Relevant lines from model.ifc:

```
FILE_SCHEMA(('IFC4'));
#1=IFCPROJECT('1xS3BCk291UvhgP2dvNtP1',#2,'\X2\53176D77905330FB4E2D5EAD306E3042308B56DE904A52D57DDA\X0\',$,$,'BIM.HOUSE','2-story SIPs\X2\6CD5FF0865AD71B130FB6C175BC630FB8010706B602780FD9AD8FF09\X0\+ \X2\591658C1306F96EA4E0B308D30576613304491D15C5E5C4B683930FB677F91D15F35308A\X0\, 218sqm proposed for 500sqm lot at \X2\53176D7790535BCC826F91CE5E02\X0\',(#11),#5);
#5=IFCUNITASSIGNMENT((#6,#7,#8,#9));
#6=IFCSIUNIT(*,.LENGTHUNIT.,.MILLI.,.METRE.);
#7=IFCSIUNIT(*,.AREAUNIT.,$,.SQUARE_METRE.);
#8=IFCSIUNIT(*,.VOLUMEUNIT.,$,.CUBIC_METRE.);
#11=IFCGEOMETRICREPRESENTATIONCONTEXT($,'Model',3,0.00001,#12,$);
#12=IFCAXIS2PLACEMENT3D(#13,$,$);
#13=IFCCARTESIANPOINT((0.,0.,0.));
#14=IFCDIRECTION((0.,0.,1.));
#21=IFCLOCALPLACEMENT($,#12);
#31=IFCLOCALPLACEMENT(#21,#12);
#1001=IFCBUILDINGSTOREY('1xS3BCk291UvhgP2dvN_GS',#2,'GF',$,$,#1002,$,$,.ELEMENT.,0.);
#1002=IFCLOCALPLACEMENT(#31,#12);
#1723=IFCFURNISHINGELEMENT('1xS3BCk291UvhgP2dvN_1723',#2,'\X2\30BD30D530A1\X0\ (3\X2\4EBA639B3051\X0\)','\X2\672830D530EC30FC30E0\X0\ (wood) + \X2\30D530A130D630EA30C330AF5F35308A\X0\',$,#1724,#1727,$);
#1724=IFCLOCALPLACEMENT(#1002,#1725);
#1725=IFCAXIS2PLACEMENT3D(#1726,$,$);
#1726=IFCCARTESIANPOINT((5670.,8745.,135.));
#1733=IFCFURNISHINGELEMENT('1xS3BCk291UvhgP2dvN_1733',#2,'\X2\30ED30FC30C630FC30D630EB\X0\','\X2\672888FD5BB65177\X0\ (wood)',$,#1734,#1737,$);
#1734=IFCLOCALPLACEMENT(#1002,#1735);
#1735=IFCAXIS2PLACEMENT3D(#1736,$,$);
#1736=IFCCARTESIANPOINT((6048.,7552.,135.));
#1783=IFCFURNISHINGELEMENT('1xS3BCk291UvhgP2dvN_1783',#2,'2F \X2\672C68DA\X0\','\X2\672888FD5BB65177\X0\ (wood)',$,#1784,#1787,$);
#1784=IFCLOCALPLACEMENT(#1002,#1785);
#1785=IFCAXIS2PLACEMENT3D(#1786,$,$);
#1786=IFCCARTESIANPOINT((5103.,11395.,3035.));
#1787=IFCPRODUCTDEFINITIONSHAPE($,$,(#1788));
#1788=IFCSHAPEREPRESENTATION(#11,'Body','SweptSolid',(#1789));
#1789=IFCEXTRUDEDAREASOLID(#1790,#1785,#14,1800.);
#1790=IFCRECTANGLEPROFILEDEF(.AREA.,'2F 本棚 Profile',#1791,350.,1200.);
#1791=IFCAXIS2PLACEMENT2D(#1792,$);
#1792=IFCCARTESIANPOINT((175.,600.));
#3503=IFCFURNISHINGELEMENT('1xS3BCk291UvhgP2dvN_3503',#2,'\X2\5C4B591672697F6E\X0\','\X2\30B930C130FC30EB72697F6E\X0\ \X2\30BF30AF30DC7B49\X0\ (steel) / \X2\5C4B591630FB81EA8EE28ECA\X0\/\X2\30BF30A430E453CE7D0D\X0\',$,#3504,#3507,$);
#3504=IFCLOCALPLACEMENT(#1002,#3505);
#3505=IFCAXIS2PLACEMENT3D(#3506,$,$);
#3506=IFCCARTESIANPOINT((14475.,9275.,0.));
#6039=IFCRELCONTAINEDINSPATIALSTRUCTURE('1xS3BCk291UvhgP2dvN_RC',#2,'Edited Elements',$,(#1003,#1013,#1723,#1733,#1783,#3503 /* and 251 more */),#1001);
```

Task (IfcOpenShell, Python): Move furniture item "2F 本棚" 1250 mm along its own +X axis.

```python
import ifcopenshell
import ifcopenshell.api.geometry
import ifcopenshell.util.placement
import ifcopenshell.util.unit

model = ifcopenshell.open("model.ifc")
unit_scale = ifcopenshell.util.unit.calculate_unit_scale(model)

item = model.by_id(1783)
matrix = ifcopenshell.util.placement.get_local_placement(item.ObjectPlacement)
matrix[:3, 3] += matrix[:3, 0] * 1.25 / unit_scale
ifcopenshell.api.geometry.edit_object_placement(model, product=item, matrix=matrix, is_si=False)

print(ifcopenshell.util.placement.get_local_placement(item.ObjectPlacement).round(3) + 0.0)

model.write("model_edited.ifc")
```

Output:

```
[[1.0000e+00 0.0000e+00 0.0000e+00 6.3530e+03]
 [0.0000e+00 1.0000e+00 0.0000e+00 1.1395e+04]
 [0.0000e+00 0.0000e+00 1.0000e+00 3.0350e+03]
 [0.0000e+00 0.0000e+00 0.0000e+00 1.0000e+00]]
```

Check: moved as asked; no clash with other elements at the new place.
